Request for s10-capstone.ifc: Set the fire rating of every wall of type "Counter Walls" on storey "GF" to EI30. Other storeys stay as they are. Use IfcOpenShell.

First a look at what the model holds.

```python
import ifcopenshell
import ifcopenshell.util.element

model = ifcopenshell.open("s10-capstone.ifc")
print(model.schema)
storey = next(s for s in model.by_type("IfcBuildingStorey") if s.Name == "GF")
walls = [e for e in ifcopenshell.util.element.get_decomposition(storey) if e.is_a("IfcWall")]
seen = {}
for e in walls:
    element_type = ifcopenshell.util.element.get_type(e)
    key = (element_type.Name if element_type != e and element_type else None, ifcopenshell.util.element.get_pset(e, "Pset_WallCommon", "FireRating"))
    seen[key] = seen.get(key, 0) + 1
for (name, value), count in sorted(seen.items(), key=str):
    print(count, "x", name, "|", value)
```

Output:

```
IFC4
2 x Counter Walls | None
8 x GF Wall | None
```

```python
import ifcopenshell
import ifcopenshell.api.pset
import ifcopenshell.util.element

model = ifcopenshell.open("s10-capstone.ifc")

storey = next(s for s in model.by_type("IfcBuildingStorey") if s.Name == "GF")
walls = [e for e in ifcopenshell.util.element.get_decomposition(storey) if e.is_a("IfcWall")]

count = 0
for e in walls:
    element_type = ifcopenshell.util.element.get_type(e)
    if element_type in (None, e) or element_type.Name != "Counter Walls":
        continue
    # add_pset returns the element's existing set when there is one.
    pset = ifcopenshell.api.pset.add_pset(model, product=e, name="Pset_WallCommon")
    ifcopenshell.api.pset.edit_pset(model, pset=pset, properties={"FireRating": "EI30"})
    count += 1

print(count, "walls updated")

model.write("s10-capstone-out.ifc")
```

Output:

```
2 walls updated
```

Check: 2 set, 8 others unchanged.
